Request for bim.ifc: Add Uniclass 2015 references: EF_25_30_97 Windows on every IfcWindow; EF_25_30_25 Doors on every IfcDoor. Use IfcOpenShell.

First a look at what the model holds.

```python
import ifcopenshell

model = ifcopenshell.open("bim.ifc")
print(model.schema)
print("classifications:", [c.Name for c in model.by_type("IfcClassification")])
for ifc_class in ("IfcDoor", "IfcRoof", "IfcStair", "IfcWall", "IfcWindow"):
    print(ifc_class, len(model.by_type(ifc_class)))
```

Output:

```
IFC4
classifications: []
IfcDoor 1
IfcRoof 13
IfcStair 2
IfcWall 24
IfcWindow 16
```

```python
import ifcopenshell
import ifcopenshell.api.classification

model = ifcopenshell.open("bim.ifc")

system = ifcopenshell.api.classification.add_classification(model, classification="Uniclass 2015")

codes = {
    "IfcWindow": ("EF_25_30_97", "Windows"),
    "IfcDoor": ("EF_25_30_25", "Doors"),
}
for ifc_class, (code, name) in codes.items():
    products = model.by_type(ifc_class)
    ifcopenshell.api.classification.add_reference(
        model, products=products, classification=system, identification=code, name=name
    )
    print(code, len(products))

model.write("bim_v2.ifc")
```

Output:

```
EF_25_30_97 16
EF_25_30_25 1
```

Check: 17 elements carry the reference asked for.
